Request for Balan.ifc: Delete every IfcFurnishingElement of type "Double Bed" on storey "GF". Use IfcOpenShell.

First a look at what the model holds.

```python
import ifcopenshell
import ifcopenshell.util.element

model = ifcopenshell.open("Balan.ifc")
print(model.schema)
storey = next(s for s in model.by_type("IfcBuildingStorey") if s.Name == "GF")
furniture = [e for e in ifcopenshell.util.element.get_decomposition(storey) if e.is_a("IfcFurnishingElement")]
seen = {}
for e in furniture:
    element_type = ifcopenshell.util.element.get_type(e)
    name = element_type.Name if element_type not in (None, e) else None
    seen[name] = seen.get(name, 0) + 1
for name, count in sorted(seen.items(), key=str):
    print(count, "x", name)
```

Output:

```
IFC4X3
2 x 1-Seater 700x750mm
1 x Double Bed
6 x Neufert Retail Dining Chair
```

```python
import ifcopenshell
import ifcopenshell.api.root
import ifcopenshell.util.element

model = ifcopenshell.open("Balan.ifc")

storey = next(s for s in model.by_type("IfcBuildingStorey") if s.Name == "GF")
furniture = [e for e in ifcopenshell.util.element.get_decomposition(storey) if e.is_a("IfcFurnishingElement")]
targets = [e for e in furniture if (t := ifcopenshell.util.element.get_type(e)) not in (None, e) and t.Name == "Double Bed"]

for e in targets:
    ifcopenshell.api.root.remove_product(model, product=e)
print(len(targets), "removed")

model.write("Balan_edited.ifc")
```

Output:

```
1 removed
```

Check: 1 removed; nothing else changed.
